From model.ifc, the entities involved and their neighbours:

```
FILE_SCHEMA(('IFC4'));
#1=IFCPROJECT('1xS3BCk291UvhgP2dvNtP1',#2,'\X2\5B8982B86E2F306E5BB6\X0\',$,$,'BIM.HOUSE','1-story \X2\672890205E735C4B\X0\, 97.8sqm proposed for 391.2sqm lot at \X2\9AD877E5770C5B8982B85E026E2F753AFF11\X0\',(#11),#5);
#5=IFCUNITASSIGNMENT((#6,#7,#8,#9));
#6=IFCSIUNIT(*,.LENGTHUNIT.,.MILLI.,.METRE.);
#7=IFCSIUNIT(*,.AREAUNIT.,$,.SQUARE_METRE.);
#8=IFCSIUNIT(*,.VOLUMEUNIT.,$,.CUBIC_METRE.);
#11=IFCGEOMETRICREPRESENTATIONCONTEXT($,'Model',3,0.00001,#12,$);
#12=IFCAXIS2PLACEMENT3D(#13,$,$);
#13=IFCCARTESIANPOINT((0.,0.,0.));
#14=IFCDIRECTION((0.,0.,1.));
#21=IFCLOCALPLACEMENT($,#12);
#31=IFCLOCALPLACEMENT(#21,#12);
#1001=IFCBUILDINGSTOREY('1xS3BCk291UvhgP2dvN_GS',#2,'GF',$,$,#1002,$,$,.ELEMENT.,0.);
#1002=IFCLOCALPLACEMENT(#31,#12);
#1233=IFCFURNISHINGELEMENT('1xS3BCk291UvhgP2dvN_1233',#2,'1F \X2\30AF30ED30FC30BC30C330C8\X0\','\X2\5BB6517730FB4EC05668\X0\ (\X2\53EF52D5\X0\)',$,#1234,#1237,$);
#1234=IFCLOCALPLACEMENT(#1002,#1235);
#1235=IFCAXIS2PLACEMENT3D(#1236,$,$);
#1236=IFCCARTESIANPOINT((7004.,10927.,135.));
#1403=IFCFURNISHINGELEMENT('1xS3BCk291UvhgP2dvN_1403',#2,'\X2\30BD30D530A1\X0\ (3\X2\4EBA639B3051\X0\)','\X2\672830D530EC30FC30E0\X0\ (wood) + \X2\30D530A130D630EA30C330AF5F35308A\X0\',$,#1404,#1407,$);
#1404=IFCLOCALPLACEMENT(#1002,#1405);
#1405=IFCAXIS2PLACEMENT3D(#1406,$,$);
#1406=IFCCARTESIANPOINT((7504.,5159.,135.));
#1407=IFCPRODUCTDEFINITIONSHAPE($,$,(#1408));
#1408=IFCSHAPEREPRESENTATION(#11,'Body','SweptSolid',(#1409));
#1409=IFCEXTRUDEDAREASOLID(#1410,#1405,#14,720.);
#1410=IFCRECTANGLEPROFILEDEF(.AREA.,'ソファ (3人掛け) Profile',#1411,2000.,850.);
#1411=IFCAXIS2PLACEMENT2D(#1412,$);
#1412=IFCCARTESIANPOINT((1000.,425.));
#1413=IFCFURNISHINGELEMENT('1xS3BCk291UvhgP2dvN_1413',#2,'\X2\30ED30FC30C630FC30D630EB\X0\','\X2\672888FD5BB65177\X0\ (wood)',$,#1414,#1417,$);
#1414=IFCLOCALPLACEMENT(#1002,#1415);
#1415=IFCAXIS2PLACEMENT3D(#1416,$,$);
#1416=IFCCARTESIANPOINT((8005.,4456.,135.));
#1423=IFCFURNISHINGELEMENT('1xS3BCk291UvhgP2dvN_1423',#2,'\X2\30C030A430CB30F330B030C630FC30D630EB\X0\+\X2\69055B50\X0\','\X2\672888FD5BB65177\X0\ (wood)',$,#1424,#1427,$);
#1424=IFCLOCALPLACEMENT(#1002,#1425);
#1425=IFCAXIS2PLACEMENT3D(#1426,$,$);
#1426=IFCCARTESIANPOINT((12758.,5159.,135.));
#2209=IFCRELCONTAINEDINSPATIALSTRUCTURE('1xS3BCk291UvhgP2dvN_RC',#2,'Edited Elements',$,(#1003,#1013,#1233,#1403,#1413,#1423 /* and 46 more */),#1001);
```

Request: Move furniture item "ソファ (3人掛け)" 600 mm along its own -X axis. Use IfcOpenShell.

```python
import ifcopenshell
import ifcopenshell.api.geometry
import ifcopenshell.util.placement
import ifcopenshell.util.unit

model = ifcopenshell.open("model.ifc")
unit_scale = ifcopenshell.util.unit.calculate_unit_scale(model)

item = model.by_guid("1xS3BCk291UvhgP2dvN_1403")
matrix = ifcopenshell.util.placement.get_local_placement(item.ObjectPlacement)
matrix[:3, 3] -= matrix[:3, 0] * 0.6 / unit_scale
ifcopenshell.api.geometry.edit_object_placement(model, product=item, matrix=matrix, is_si=False)

print(ifcopenshell.util.placement.get_local_placement(item.ObjectPlacement).round(3) + 0.0)

model.write("model_edited.ifc")
```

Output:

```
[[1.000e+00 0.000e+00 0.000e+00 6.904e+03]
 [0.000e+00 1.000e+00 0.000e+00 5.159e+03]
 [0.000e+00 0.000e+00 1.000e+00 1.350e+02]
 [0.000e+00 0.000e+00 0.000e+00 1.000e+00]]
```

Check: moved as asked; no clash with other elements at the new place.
